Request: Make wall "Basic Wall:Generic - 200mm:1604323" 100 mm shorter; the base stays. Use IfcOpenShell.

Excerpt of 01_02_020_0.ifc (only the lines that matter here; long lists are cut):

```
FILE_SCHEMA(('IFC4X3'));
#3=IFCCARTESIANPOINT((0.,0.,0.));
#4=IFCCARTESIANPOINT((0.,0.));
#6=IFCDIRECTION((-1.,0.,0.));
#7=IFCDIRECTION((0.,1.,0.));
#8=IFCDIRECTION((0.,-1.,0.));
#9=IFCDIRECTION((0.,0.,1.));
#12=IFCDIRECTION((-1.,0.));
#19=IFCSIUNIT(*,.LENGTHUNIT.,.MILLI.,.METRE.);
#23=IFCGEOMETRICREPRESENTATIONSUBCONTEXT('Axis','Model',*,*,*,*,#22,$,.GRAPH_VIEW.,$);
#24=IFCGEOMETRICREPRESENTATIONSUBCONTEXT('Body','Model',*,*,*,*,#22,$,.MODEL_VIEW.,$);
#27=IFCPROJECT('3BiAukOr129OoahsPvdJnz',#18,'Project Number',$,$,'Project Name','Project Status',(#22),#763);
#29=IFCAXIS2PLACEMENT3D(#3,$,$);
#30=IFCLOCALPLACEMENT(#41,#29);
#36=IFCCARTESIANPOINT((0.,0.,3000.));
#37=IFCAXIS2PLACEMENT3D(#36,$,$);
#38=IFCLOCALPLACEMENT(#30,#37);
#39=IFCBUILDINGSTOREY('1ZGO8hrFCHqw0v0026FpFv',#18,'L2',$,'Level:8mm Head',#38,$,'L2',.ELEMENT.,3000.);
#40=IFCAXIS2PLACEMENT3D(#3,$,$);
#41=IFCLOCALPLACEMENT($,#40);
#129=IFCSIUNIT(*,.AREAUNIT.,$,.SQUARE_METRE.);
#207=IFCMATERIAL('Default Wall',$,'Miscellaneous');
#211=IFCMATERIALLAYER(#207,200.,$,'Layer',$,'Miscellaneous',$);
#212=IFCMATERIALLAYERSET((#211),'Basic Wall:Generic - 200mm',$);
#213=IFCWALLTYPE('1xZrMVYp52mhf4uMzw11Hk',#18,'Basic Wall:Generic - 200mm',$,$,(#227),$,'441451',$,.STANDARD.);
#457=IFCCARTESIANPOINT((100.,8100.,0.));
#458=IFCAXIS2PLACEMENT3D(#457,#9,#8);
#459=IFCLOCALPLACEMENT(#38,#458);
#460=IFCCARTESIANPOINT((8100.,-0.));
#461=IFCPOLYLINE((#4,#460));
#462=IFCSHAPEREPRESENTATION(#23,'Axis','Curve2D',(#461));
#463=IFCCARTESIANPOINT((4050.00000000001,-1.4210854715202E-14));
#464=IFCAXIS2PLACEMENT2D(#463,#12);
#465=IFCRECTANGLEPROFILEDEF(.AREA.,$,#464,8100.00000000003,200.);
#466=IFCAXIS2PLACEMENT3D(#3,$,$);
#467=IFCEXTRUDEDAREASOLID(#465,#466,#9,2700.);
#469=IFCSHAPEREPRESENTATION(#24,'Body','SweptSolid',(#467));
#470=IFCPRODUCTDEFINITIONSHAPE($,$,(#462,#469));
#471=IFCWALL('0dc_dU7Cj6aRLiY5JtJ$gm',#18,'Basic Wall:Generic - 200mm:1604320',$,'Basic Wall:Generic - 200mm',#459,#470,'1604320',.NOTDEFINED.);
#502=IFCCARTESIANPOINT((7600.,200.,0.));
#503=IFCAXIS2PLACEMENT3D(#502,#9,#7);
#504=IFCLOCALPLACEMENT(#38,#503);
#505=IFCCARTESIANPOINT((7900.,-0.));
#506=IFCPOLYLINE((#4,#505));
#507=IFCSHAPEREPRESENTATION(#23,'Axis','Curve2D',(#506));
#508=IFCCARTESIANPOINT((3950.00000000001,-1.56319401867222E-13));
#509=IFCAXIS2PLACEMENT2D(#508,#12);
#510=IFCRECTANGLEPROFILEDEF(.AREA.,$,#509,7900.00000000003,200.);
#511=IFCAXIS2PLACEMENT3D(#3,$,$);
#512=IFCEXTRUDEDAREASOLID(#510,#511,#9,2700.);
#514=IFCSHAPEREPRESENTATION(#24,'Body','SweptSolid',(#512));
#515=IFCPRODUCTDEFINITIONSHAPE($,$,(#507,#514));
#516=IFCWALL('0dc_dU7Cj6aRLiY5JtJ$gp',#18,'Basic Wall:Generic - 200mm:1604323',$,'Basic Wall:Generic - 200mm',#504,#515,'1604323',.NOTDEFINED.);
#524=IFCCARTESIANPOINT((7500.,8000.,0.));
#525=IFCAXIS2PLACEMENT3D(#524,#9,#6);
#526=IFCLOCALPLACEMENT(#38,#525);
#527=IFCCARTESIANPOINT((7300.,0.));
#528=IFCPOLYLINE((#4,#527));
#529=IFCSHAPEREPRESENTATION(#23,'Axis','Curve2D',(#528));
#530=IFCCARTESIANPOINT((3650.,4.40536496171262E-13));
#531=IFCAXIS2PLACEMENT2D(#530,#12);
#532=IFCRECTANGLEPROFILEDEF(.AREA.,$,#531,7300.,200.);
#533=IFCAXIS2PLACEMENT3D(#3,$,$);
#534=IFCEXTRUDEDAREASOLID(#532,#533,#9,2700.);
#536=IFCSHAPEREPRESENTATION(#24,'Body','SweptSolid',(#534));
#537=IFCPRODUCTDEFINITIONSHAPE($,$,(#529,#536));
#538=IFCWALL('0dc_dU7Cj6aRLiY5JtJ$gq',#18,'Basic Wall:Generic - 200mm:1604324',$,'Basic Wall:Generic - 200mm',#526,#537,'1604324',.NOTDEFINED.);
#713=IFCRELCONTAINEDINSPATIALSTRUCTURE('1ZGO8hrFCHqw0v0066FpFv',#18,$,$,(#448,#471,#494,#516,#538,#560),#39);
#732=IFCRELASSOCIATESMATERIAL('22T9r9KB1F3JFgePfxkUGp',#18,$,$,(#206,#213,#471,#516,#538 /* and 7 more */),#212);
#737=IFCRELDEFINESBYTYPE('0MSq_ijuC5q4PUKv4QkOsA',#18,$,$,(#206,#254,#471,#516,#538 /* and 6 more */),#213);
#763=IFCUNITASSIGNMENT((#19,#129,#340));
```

```python
import ifcopenshell
import ifcopenshell.geom
import ifcopenshell.util.representation
import ifcopenshell.util.shape
import ifcopenshell.util.unit

model = ifcopenshell.open("01_02_020_0.ifc")
unit_scale = ifcopenshell.util.unit.calculate_unit_scale(model)
settings = ifcopenshell.geom.settings()


def volume(element):
    """Net volume in cubic metres, openings subtracted."""
    shape = ifcopenshell.geom.create_shape(settings, element)
    return ifcopenshell.util.shape.get_volume(shape.geometry)


wall = model.by_guid("0dc_dU7Cj6aRLiY5JtJ$gp")
before = volume(wall)

body = ifcopenshell.util.representation.get_representation(wall, "Model", "Body")
solid = body.Items[0]
old_height = solid.Depth
solid.Depth -= 0.1 / unit_scale
after = volume(wall)

print(f"height {old_height:g} -> {solid.Depth:g}, volume {before:.3f} -> {after:.3f} m3")

model.write("01_02_020_0_updated.ifc")
```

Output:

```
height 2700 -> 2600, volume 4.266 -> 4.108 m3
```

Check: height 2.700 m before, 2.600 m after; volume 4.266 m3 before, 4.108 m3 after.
